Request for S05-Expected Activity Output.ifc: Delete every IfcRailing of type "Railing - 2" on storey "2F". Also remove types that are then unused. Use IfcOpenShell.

First a look at what the model holds.

```python
import ifcopenshell
import ifcopenshell.util.element

model = ifcopenshell.open("S05-Expected Activity Output.ifc")
print(model.schema)
storey = next(s for s in model.by_type("IfcBuildingStorey") if s.Name == "2F")
railings = [e for e in ifcopenshell.util.element.get_decomposition(storey) if e.is_a("IfcRailing")]
seen = {}
for e in railings:
    element_type = ifcopenshell.util.element.get_type(e)
    name = element_type.Name if element_type not in (None, e) else None
    seen[name] = seen.get(name, 0) + 1
for name, count in sorted(seen.items(), key=str):
    print(count, "x", name)
```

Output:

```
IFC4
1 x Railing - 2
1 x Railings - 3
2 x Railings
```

```python
import ifcopenshell
import ifcopenshell.api.root
import ifcopenshell.util.element

model = ifcopenshell.open("S05-Expected Activity Output.ifc")

storey = next(s for s in model.by_type("IfcBuildingStorey") if s.Name == "2F")
railings = [e for e in ifcopenshell.util.element.get_decomposition(storey) if e.is_a("IfcRailing")]
targets = [e for e in railings if (t := ifcopenshell.util.element.get_type(e)) not in (None, e) and t.Name == "Railing - 2"]
types = {ifcopenshell.util.element.get_type(e) for e in targets} - {None, *targets}

for e in targets:
    ifcopenshell.api.root.remove_product(model, product=e)
print(len(targets), "removed")

unused = [t for t in types if not ifcopenshell.util.element.get_types(t)]
for t in unused:
    ifcopenshell.api.root.remove_product(model, product=t)
print(len(unused), "unused types removed")

model.write("S05-Expected Activity Output_edited.ifc")
```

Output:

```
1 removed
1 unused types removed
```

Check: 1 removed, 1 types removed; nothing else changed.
